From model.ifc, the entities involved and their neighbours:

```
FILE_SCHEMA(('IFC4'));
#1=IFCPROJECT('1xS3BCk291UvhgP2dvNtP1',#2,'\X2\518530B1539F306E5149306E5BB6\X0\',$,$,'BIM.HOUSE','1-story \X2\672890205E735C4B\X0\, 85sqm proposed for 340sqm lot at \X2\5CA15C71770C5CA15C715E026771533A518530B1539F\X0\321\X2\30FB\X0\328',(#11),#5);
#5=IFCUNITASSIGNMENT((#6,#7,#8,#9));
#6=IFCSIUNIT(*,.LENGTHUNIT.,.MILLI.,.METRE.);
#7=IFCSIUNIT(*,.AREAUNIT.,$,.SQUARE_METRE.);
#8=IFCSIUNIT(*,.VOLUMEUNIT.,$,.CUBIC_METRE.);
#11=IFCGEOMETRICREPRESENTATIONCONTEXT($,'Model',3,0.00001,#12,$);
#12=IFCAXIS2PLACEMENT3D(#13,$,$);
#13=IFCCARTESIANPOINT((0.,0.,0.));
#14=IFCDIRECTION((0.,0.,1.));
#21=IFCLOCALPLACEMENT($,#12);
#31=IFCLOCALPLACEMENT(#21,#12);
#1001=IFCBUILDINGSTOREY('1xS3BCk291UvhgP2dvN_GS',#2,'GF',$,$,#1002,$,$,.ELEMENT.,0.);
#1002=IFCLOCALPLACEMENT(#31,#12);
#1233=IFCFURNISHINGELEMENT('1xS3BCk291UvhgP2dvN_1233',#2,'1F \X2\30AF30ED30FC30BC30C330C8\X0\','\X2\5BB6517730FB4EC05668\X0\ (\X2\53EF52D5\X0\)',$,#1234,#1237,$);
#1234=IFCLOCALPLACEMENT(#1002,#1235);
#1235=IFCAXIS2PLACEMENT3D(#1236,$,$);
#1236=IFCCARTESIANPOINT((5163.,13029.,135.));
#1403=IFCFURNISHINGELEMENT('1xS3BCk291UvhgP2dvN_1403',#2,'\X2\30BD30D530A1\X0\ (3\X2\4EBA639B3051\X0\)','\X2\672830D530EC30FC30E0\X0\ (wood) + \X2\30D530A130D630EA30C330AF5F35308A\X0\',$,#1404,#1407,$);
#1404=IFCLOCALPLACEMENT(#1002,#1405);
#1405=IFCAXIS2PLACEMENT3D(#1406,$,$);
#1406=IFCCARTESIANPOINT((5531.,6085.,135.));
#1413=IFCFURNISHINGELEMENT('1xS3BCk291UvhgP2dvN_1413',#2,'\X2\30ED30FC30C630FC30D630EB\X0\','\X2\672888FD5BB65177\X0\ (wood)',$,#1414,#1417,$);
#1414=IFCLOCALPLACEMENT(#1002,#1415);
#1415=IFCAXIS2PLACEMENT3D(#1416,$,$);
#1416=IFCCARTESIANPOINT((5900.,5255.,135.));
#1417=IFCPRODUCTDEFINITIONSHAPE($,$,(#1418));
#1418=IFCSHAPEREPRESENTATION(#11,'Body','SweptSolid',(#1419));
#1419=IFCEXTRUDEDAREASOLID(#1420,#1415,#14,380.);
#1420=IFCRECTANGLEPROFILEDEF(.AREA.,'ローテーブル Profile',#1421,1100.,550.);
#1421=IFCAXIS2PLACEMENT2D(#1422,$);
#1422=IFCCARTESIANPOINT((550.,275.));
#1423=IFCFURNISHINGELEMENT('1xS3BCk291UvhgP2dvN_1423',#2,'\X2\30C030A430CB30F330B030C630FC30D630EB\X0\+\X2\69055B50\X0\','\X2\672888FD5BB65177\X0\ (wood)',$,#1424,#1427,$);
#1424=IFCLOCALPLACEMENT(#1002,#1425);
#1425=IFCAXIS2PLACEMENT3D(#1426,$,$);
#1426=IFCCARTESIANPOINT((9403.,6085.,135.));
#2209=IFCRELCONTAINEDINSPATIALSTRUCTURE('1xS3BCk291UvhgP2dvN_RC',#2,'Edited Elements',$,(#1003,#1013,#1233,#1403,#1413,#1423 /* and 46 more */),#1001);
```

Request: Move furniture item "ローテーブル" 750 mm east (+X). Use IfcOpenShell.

```python
import ifcopenshell
import ifcopenshell.api.geometry
import ifcopenshell.util.placement
import ifcopenshell.util.unit

model = ifcopenshell.open("model.ifc")
unit_scale = ifcopenshell.util.unit.calculate_unit_scale(model)

item = model.by_guid("1xS3BCk291UvhgP2dvN_1413")
matrix = ifcopenshell.util.placement.get_local_placement(item.ObjectPlacement)
matrix[0, 3] += 0.75 / unit_scale
ifcopenshell.api.geometry.edit_object_placement(model, product=item, matrix=matrix, is_si=False)

print(ifcopenshell.util.placement.get_local_placement(item.ObjectPlacement).round(3) + 0.0)

model.write("model_updated.ifc")
```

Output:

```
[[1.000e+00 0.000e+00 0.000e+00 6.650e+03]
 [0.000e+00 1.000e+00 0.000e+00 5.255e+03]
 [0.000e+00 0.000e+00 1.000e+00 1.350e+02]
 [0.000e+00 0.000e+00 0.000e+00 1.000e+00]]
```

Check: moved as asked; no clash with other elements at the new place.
